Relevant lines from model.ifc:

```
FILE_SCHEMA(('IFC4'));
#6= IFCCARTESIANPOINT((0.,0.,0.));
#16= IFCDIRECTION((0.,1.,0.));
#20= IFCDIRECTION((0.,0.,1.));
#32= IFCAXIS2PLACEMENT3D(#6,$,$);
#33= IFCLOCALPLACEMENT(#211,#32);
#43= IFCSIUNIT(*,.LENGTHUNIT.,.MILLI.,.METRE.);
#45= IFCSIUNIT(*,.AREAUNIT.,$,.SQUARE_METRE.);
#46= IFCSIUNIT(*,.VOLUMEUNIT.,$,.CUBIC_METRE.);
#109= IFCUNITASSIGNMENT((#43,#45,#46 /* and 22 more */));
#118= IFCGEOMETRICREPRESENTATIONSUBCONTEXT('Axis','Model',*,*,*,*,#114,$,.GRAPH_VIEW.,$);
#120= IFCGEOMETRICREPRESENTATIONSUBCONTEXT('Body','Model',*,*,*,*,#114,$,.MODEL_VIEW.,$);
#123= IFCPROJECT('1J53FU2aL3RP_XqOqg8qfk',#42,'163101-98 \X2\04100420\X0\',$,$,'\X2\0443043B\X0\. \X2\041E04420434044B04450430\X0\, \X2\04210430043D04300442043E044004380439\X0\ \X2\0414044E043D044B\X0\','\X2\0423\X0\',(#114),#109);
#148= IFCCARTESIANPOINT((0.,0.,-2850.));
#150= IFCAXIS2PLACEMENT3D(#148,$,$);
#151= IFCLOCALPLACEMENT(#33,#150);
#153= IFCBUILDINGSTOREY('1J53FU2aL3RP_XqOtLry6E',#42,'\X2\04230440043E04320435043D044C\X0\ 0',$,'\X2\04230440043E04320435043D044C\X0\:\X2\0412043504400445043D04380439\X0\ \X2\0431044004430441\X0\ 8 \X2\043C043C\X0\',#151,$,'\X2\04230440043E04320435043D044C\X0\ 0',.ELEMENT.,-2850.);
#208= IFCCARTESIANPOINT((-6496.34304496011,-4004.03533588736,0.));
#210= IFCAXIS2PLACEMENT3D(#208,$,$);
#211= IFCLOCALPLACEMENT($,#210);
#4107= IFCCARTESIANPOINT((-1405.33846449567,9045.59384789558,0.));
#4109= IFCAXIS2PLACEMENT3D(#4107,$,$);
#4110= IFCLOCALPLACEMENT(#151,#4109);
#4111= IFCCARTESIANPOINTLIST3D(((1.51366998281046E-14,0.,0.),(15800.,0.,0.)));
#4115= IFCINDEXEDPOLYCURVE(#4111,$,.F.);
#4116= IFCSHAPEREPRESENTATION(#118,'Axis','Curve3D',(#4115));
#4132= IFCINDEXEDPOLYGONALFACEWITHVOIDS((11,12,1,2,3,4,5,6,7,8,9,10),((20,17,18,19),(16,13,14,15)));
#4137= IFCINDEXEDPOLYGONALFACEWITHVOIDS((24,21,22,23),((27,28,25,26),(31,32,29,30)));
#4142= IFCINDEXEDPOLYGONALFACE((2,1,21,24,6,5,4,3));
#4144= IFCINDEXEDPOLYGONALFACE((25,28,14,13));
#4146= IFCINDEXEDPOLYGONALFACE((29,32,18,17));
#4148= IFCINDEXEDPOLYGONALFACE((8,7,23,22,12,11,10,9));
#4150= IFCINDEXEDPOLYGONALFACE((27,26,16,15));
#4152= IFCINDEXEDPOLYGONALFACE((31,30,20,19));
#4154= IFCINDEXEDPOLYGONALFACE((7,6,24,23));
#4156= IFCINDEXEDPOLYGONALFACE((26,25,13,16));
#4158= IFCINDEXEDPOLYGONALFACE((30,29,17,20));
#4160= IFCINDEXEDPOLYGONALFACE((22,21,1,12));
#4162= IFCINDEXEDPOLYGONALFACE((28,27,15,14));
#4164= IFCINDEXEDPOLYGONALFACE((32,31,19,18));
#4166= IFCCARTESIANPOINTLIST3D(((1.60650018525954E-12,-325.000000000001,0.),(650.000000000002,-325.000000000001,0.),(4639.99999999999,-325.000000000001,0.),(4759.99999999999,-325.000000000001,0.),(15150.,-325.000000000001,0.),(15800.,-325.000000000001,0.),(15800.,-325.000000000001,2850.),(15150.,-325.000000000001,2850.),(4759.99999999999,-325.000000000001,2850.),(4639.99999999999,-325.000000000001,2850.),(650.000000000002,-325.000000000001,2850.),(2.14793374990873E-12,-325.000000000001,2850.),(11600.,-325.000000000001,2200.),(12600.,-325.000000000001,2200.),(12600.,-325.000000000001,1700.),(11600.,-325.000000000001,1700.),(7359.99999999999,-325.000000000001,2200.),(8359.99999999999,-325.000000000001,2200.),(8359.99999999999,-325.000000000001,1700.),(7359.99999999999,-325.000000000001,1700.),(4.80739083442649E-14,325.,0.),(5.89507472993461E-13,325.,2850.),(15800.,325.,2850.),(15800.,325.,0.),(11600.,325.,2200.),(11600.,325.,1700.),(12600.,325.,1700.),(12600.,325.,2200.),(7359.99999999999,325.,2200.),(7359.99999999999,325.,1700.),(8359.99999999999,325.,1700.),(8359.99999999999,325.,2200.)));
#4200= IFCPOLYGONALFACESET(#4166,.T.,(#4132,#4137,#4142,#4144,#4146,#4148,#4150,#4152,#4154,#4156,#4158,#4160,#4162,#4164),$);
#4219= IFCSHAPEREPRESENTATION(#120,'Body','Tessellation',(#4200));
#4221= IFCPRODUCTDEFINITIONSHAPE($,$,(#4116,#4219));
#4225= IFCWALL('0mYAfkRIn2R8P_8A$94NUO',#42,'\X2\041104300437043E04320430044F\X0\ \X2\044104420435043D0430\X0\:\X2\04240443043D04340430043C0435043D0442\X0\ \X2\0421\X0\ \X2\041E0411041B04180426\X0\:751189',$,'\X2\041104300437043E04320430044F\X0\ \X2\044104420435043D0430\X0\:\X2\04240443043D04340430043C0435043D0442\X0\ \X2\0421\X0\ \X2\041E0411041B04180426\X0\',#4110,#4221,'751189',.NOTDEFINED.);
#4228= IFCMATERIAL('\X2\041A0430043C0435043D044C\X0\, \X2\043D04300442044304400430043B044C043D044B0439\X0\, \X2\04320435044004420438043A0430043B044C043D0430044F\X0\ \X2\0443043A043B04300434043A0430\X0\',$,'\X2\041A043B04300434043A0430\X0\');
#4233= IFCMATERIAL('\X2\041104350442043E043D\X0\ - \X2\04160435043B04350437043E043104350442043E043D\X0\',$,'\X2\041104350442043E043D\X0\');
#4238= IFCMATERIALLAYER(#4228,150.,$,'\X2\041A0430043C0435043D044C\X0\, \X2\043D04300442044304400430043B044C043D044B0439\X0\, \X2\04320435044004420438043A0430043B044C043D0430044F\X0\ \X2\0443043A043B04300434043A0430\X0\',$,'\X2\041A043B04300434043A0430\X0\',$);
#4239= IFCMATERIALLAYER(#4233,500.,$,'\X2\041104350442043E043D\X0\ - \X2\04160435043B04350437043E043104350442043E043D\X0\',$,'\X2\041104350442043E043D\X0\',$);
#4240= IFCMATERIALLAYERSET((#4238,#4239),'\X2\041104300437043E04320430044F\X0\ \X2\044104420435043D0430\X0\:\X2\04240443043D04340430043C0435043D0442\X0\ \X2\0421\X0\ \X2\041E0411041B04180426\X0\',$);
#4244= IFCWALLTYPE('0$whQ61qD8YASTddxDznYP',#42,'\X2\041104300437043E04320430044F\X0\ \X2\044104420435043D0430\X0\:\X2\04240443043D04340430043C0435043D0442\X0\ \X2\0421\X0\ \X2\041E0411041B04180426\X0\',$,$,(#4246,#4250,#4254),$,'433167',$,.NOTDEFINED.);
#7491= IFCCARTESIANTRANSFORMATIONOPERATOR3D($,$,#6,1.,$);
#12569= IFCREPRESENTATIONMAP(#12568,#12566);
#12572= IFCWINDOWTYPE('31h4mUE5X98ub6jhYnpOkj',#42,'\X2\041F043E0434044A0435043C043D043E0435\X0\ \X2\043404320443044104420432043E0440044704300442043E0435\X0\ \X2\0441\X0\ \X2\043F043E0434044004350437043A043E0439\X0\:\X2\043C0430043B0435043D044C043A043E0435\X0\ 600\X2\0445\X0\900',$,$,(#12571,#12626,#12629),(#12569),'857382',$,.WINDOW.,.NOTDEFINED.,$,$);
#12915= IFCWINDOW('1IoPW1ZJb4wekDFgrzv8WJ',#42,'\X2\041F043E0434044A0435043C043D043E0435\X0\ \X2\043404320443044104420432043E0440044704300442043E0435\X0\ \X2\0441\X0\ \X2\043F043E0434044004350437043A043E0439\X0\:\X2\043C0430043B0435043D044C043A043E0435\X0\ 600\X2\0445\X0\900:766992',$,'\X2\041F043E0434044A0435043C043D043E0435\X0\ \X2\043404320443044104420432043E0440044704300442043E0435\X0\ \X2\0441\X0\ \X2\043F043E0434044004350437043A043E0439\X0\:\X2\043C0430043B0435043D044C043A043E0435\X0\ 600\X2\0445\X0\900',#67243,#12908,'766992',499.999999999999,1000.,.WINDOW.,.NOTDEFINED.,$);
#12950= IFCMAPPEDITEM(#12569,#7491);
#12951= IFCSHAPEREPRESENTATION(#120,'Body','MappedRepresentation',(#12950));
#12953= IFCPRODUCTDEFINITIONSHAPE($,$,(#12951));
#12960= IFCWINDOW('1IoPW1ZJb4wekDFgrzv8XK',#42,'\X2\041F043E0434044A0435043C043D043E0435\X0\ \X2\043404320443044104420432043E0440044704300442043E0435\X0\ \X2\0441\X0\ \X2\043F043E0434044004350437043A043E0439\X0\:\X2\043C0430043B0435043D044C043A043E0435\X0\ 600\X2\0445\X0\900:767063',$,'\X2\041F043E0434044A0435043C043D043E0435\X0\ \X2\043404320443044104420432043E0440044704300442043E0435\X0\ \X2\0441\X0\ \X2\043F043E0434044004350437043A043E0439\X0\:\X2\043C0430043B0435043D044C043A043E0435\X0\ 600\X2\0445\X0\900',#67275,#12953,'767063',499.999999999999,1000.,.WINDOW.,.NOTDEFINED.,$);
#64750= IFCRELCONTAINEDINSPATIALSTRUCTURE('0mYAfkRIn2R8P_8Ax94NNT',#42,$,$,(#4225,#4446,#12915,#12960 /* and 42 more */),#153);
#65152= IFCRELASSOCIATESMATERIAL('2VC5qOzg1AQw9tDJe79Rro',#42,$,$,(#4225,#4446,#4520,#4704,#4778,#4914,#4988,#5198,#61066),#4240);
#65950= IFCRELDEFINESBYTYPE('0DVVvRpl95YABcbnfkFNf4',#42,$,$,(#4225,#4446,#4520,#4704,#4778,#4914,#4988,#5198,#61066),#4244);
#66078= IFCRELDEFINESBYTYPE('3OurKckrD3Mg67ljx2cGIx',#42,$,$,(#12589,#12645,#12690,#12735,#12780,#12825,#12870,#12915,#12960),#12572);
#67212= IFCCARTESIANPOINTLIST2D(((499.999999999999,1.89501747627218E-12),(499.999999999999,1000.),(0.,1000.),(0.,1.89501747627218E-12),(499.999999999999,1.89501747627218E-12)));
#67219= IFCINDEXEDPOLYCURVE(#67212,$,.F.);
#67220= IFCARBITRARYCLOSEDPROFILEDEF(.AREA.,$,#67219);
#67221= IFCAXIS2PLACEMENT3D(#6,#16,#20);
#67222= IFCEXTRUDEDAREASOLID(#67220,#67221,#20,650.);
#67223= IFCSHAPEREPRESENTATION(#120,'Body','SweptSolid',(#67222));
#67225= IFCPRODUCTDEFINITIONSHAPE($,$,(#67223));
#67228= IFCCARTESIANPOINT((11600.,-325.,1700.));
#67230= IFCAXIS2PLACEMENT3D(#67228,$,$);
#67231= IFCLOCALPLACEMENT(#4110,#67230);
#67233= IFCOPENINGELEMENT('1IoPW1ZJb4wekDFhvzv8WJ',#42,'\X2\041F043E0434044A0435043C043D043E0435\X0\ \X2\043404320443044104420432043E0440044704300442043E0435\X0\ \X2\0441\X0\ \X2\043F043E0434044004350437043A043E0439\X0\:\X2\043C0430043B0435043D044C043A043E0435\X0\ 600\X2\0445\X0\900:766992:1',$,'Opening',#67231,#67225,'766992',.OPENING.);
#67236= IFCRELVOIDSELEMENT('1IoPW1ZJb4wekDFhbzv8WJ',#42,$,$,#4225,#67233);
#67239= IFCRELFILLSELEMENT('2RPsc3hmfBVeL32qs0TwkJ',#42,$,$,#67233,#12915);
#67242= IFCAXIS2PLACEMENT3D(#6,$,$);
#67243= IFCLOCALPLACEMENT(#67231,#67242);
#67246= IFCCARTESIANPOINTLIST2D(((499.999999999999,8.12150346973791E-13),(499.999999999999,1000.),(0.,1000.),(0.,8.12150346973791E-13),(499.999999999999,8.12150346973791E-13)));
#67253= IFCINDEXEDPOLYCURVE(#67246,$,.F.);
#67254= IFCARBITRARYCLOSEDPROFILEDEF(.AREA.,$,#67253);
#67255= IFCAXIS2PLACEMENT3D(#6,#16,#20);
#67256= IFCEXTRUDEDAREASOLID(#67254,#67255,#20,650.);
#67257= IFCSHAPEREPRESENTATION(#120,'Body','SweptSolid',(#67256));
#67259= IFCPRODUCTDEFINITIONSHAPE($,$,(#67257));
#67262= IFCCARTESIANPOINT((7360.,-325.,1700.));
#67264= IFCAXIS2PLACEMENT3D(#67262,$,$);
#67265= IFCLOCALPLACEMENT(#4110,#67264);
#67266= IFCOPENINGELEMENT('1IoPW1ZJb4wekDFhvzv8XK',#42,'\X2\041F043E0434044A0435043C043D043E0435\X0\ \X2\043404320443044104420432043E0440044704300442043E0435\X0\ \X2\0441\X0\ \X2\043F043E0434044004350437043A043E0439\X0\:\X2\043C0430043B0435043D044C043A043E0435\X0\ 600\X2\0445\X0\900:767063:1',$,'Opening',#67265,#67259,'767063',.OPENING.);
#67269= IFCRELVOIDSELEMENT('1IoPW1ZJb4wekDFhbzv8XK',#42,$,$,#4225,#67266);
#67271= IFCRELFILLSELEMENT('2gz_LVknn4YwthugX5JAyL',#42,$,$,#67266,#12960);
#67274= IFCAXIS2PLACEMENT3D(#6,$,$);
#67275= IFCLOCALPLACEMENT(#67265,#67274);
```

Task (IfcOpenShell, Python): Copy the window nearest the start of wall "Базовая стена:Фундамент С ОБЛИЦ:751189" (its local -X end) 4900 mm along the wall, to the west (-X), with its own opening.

```python
import ifcopenshell
import ifcopenshell.api.feature
import ifcopenshell.api.geometry
import ifcopenshell.api.root
import ifcopenshell.geom
import ifcopenshell.util.element
import ifcopenshell.util.placement
import ifcopenshell.util.shape

model = ifcopenshell.open("model.ifc")
settings = ifcopenshell.geom.settings()


def volume(element):
    """Net volume in cubic metres, openings subtracted."""
    shape = ifcopenshell.geom.create_shape(settings, element)
    return ifcopenshell.util.shape.get_volume(shape.geometry)


def reuse_history(source, copy):
    """copy_class also copies each property set's owner history, people and application; keep the originals."""
    for rel in copy.IsDefinedBy:
        if rel.is_a("IfcRelDefinesByProperties") and (history := rel.RelatingPropertyDefinition.OwnerHistory):
            rel.RelatingPropertyDefinition.OwnerHistory = source.OwnerHistory
            ifcopenshell.util.element.remove_deep2(model, history)


window = model.by_guid("1IoPW1ZJb4wekDFgrzv8XK")
opening = window.FillsVoids[0].RelatingOpeningElement
wall = opening.VoidsElements[0].RelatingBuildingElement
before = volume(wall)
shift = ifcopenshell.util.placement.get_local_placement(wall.ObjectPlacement)[:3, 0] * -4900.0

# copy_class copies the void relationship, type, container and properties, but no geometry.
new_opening = ifcopenshell.api.root.copy_class(model, product=opening)
new_opening.Representation = ifcopenshell.util.element.copy_deep(
    model, opening.Representation, exclude=["IfcGeometricRepresentationContext", "IfcRepresentationMap"]
)
new_opening.Name = "Подъемное двустворчатое с подрезкой:маленькое 600х900"
new_opening.Tag = None
new_window = ifcopenshell.api.root.copy_class(model, product=window)
new_window.Representation = ifcopenshell.util.element.copy_deep(
    model, window.Representation, exclude=["IfcGeometricRepresentationContext", "IfcRepresentationMap"]
)
new_window.Name = "Подъемное двустворчатое с подрезкой:маленькое 600х900"
new_window.Tag = None
reuse_history(window, new_window)
ifcopenshell.api.feature.add_filling(model, opening=new_opening, element=new_window)

for old, new in ((opening, new_opening), (window, new_window)):
    matrix = ifcopenshell.util.placement.get_local_placement(old.ObjectPlacement)
    matrix[:3, 3] += shift
    ifcopenshell.api.geometry.edit_object_placement(model, product=new, matrix=matrix, is_si=False)

after = volume(wall)

print(f"wall volume {before:.3f} -> {after:.3f} m3")

model.write("model_rev.ifc")
```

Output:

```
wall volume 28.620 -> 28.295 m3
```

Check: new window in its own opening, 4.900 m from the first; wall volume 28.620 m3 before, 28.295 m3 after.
